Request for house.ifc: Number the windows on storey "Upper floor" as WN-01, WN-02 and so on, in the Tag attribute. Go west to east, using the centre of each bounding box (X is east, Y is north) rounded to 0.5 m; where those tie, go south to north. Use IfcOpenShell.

First a look at what the model holds.

```python
import ifcopenshell
import ifcopenshell.util.element
import ifcopenshell.util.placement

model = ifcopenshell.open("house.ifc")
print(model.schema)
storey = next(s for s in model.by_type("IfcBuildingStorey") if s.Name == "Upper floor")
windows = [e for e in ifcopenshell.util.element.get_decomposition(storey) if e.is_a("IfcWindow")]
for e in sorted(windows, key=lambda e: e.id()):
    origin = ifcopenshell.util.placement.get_local_placement(e.ObjectPlacement)[:3, 3]
    print(e.id(), e.Tag, e.Name, origin.round(2) + 0.0, sep=" | ")
```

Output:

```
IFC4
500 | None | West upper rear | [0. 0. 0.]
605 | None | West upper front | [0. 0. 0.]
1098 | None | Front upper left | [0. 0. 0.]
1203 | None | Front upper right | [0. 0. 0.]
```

```python
import ifcopenshell
import ifcopenshell.geom
import ifcopenshell.util.element
import ifcopenshell.util.shape

model = ifcopenshell.open("house.ifc")
settings = ifcopenshell.geom.settings()
settings.set("use-world-coords", True)


def centre(element):
    shape = ifcopenshell.geom.create_shape(settings, element)
    return ifcopenshell.util.shape.get_bbox_centroid(shape.geometry)


storey = next(s for s in model.by_type("IfcBuildingStorey") if s.Name == "Upper floor")
windows = [e for e in ifcopenshell.util.element.get_decomposition(storey) if e.is_a("IfcWindow")]

# Insertion points can sit at a corner or the storey origin, so sort by the geometry (in metres).
centres = {e: centre(e) for e in windows}
windows.sort(key=lambda e: (round(centres[e][0] / 0.5), centres[e][1]))

for i, e in enumerate(windows, start=1):
    number = f"WN-{i:02d}"
    e.Tag = number
    print(e.id(), number)

model.write("house_edited.ifc")
```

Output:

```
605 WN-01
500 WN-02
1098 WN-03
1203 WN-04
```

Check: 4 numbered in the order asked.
